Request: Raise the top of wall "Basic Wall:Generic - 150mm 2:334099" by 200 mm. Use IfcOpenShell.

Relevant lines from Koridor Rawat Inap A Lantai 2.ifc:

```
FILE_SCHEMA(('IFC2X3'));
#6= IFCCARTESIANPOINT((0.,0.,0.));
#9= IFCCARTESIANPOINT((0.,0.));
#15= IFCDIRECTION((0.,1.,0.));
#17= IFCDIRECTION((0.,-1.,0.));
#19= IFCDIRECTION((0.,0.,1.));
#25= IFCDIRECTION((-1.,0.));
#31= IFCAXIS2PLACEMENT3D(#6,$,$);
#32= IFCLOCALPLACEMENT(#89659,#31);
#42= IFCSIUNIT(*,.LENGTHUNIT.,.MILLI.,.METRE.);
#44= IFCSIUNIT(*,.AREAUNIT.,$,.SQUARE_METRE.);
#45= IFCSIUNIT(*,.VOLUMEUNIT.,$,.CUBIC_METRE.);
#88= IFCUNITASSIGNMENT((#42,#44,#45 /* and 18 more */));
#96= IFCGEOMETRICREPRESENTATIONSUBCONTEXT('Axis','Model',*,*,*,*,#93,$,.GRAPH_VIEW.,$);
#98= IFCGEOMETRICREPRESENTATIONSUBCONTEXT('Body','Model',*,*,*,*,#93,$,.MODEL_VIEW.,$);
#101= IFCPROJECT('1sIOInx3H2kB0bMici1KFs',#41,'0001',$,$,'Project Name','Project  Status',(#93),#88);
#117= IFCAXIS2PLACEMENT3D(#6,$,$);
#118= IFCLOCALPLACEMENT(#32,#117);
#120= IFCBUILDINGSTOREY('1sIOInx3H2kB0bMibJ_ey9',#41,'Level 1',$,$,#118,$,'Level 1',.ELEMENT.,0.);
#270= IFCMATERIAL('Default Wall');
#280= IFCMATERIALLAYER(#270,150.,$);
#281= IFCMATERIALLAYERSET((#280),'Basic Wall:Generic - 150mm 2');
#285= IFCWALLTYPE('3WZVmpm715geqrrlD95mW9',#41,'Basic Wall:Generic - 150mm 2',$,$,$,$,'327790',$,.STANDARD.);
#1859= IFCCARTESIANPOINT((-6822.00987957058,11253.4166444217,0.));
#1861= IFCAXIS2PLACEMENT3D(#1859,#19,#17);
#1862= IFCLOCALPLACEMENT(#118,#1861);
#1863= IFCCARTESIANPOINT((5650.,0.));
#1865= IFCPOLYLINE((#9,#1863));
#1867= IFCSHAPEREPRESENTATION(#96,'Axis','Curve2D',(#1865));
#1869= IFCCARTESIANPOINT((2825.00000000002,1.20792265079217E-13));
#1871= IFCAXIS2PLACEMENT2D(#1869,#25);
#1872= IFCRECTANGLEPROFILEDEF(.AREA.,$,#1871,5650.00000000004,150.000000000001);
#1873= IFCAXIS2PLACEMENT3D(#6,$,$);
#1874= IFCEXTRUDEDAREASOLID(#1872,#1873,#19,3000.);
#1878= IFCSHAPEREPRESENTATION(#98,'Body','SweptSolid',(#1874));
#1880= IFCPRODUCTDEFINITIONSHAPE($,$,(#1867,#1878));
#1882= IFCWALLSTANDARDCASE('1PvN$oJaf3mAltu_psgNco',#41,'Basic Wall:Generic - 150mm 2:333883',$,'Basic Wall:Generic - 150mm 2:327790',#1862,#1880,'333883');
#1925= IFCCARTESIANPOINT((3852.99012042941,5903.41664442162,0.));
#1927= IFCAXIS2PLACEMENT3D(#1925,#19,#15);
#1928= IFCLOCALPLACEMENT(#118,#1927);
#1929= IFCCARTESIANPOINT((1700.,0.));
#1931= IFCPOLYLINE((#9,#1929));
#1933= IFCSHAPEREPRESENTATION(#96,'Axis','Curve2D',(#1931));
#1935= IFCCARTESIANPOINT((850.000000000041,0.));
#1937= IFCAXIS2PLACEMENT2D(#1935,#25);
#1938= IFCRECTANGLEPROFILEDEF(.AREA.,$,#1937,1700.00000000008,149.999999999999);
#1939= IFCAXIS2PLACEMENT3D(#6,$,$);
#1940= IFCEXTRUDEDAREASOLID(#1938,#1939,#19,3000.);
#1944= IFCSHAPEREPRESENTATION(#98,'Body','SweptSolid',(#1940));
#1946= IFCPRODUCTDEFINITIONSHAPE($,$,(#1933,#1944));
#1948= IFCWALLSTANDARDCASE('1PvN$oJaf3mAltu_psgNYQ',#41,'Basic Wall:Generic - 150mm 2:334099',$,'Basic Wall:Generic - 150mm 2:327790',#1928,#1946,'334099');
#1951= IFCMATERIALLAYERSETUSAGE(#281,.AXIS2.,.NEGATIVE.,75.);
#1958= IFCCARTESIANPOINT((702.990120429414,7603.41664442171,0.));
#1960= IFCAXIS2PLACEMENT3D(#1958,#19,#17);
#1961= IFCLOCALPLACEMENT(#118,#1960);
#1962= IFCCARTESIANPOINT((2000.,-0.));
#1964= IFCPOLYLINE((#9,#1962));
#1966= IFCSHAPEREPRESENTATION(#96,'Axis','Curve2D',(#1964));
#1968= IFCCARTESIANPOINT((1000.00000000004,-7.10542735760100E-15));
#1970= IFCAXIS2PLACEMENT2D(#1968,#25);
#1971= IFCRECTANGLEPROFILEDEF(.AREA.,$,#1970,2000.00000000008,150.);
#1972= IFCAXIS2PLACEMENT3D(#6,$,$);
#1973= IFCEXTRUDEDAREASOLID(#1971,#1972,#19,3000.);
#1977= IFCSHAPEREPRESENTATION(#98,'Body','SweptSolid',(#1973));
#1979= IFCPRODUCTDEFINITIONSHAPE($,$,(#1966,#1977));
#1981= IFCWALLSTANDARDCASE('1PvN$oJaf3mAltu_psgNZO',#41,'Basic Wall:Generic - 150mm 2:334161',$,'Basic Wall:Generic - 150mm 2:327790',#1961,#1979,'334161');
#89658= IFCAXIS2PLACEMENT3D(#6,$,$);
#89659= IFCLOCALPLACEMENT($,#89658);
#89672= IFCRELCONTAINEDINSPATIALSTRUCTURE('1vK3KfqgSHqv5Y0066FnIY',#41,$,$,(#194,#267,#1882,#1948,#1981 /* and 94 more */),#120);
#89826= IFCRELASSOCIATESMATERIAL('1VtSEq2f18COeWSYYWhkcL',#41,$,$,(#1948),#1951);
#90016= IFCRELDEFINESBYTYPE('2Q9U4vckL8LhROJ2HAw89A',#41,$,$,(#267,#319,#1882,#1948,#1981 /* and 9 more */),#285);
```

```python
import ifcopenshell
import ifcopenshell.geom
import ifcopenshell.util.representation
import ifcopenshell.util.shape
import ifcopenshell.util.unit

model = ifcopenshell.open("Koridor Rawat Inap A Lantai 2.ifc")
unit_scale = ifcopenshell.util.unit.calculate_unit_scale(model)
settings = ifcopenshell.geom.settings()


def volume(element):
    """Net volume in cubic metres, openings subtracted."""
    shape = ifcopenshell.geom.create_shape(settings, element)
    return ifcopenshell.util.shape.get_volume(shape.geometry)


wall = model.by_guid("1PvN$oJaf3mAltu_psgNYQ")
before = volume(wall)

body = ifcopenshell.util.representation.get_representation(wall, "Model", "Body")
solid = body.Items[0]
old_height = solid.Depth
solid.Depth += 0.2 / unit_scale
after = volume(wall)

print(f"height {old_height:g} -> {solid.Depth:g}, volume {before:.3f} -> {after:.3f} m3")

model.write("Koridor Rawat Inap A Lantai 2-out.ifc")
```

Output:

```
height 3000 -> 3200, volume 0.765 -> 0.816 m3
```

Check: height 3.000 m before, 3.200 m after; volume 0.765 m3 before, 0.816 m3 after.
